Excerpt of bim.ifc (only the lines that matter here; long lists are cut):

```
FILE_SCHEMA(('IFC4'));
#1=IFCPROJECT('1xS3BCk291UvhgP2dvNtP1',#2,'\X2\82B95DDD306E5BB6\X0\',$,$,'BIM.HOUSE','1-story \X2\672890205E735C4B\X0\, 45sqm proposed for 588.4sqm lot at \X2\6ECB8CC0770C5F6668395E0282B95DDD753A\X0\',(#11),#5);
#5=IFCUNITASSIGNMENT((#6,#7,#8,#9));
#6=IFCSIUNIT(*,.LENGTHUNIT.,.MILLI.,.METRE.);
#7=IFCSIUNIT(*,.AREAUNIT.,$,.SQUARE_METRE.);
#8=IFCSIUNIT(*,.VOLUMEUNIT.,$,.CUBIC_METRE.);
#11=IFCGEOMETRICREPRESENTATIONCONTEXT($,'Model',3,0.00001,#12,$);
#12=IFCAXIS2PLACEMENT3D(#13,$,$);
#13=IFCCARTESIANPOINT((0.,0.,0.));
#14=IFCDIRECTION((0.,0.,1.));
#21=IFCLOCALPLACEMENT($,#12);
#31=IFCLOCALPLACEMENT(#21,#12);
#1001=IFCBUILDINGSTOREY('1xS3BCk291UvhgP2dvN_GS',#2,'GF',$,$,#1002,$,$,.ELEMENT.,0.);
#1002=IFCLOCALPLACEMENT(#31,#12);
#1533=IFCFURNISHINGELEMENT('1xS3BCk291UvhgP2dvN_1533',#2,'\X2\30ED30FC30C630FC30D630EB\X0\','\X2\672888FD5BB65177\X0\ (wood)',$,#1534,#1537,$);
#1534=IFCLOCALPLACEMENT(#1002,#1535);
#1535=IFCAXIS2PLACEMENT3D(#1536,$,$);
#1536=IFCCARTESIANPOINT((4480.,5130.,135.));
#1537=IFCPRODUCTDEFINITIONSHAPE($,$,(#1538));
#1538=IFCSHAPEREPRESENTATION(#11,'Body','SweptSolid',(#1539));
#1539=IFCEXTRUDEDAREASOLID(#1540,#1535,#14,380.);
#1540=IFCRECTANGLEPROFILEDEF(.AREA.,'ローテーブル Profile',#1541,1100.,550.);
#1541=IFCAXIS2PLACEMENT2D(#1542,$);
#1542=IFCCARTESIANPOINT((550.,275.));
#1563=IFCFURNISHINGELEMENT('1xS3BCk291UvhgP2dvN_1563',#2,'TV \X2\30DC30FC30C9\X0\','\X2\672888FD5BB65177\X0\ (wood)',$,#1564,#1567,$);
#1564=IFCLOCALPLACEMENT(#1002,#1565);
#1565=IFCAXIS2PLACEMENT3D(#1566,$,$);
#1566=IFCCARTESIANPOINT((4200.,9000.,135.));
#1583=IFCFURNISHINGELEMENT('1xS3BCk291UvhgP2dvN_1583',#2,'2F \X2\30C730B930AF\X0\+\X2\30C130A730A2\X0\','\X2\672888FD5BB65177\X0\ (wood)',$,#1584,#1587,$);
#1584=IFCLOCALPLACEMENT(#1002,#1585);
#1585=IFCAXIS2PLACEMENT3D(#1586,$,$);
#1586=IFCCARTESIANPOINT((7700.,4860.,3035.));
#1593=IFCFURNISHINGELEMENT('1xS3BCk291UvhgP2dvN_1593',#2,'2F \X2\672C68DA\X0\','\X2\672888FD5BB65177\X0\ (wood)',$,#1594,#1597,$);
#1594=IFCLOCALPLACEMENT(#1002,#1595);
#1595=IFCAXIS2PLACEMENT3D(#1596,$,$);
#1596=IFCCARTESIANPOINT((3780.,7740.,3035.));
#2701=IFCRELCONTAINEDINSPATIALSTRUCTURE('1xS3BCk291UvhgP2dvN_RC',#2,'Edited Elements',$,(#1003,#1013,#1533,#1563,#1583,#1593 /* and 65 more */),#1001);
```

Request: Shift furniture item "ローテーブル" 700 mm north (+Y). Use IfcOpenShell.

```python
import ifcopenshell
import ifcopenshell.api.geometry
import ifcopenshell.util.placement
import ifcopenshell.util.unit

model = ifcopenshell.open("bim.ifc")
unit_scale = ifcopenshell.util.unit.calculate_unit_scale(model)

item = model.by_guid("1xS3BCk291UvhgP2dvN_1533")
matrix = ifcopenshell.util.placement.get_local_placement(item.ObjectPlacement)
matrix[1, 3] += 0.7 / unit_scale
ifcopenshell.api.geometry.edit_object_placement(model, product=item, matrix=matrix, is_si=False)

print(ifcopenshell.util.placement.get_local_placement(item.ObjectPlacement).round(3) + 0.0)

model.write("bim_rev.ifc")
```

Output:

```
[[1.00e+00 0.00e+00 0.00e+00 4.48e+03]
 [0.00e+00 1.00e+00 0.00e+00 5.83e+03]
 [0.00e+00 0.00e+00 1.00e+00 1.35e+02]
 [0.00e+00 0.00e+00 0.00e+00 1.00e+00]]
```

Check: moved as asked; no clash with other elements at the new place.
